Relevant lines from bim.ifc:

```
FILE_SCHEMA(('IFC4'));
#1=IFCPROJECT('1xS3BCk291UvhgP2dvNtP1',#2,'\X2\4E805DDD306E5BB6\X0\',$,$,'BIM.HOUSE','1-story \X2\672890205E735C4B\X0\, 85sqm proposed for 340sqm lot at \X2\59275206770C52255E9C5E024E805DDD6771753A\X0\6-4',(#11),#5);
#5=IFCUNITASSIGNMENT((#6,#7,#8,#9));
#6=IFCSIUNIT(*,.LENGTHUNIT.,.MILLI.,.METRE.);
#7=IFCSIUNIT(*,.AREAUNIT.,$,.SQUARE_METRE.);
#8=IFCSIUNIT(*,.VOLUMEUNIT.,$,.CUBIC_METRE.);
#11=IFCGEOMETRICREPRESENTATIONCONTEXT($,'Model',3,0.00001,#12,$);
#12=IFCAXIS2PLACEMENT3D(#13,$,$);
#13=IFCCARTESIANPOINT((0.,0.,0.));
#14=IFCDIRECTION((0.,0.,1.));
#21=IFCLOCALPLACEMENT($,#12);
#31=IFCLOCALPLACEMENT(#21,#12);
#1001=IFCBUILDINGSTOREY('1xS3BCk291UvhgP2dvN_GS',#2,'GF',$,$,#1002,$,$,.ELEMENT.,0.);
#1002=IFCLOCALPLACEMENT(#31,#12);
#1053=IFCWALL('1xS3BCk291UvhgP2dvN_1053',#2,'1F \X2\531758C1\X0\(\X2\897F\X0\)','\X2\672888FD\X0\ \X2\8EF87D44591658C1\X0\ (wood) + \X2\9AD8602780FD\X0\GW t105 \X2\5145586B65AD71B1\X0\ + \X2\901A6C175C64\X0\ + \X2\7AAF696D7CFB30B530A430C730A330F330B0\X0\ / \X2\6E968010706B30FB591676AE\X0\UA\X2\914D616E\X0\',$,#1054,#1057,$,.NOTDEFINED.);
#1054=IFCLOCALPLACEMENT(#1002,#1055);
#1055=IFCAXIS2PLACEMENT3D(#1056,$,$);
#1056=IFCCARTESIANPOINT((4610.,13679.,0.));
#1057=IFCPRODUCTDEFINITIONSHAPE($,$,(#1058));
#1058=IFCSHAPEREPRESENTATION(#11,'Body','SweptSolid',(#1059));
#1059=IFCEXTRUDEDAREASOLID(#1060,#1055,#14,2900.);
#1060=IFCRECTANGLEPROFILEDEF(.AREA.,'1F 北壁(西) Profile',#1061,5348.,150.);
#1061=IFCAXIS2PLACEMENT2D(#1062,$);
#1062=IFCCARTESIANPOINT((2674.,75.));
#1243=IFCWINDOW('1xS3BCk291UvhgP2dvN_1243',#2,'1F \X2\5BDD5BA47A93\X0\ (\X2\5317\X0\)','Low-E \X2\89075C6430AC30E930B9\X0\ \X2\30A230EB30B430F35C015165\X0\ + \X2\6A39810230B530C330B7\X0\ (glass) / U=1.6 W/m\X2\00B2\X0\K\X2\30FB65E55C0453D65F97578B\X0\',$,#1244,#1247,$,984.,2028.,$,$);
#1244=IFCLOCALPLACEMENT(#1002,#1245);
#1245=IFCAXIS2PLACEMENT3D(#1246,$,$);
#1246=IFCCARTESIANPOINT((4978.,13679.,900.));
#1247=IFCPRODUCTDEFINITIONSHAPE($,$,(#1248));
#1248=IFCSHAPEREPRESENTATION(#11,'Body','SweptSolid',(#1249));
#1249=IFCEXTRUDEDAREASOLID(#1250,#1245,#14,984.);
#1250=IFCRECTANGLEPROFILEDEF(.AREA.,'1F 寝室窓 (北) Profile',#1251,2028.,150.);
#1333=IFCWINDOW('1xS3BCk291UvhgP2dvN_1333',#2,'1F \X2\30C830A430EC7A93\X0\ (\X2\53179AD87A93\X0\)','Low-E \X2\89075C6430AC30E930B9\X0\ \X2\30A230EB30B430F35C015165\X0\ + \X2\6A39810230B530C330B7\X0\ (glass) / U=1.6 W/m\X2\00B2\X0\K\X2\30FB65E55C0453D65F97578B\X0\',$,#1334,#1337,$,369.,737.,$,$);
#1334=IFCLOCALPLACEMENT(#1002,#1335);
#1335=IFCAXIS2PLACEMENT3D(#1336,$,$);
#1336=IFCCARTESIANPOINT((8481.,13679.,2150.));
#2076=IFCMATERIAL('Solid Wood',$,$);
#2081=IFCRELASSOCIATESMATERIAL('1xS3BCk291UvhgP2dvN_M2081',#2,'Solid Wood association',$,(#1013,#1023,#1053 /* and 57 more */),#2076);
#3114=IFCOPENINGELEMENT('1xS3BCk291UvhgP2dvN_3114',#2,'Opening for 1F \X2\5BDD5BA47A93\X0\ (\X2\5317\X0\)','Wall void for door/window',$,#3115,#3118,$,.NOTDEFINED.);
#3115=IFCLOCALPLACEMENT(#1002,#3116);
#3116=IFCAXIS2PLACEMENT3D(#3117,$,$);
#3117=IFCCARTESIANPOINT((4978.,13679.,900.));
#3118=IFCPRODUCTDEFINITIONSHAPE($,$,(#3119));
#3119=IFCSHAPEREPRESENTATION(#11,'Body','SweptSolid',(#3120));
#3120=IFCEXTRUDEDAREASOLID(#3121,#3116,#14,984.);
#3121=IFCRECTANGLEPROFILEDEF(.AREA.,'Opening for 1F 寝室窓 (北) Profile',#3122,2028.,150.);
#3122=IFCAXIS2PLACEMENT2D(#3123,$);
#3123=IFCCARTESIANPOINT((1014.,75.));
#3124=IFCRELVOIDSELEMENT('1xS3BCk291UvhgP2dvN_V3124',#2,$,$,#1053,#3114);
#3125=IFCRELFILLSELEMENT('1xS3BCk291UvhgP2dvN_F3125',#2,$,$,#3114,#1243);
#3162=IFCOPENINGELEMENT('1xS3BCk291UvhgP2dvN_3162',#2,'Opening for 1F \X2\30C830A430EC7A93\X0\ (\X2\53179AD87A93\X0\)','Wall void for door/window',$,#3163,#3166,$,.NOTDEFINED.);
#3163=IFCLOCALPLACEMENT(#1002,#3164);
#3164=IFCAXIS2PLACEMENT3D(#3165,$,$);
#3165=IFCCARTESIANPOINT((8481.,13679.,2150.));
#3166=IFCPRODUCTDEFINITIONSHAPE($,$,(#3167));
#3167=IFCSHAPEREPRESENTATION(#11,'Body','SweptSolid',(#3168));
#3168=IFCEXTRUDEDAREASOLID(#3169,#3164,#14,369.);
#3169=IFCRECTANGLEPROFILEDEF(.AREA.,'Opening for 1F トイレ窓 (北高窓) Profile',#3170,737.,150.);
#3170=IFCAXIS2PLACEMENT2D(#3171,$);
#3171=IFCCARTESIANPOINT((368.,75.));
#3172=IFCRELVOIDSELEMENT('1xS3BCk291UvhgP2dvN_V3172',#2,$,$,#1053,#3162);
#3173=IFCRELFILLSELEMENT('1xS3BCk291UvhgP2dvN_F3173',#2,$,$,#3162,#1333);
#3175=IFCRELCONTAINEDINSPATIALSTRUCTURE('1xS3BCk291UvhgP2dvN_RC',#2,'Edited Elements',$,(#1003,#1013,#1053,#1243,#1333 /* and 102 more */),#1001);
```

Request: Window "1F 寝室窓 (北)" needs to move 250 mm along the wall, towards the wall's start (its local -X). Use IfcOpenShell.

```python
import ifcopenshell
import ifcopenshell.api.geometry
import ifcopenshell.util.placement

model = ifcopenshell.open("bim.ifc")

window = model.by_guid("1xS3BCk291UvhgP2dvN_1243")
opening = window.FillsVoids[0].RelatingOpeningElement
wall = opening.VoidsElements[0].RelatingBuildingElement

wall_matrix = ifcopenshell.util.placement.get_local_placement(wall.ObjectPlacement)
shift = wall_matrix[:3, 0] * -250.0
before = ifcopenshell.util.placement.get_local_placement(window.ObjectPlacement)[:3, 3].copy()

# The window is not placed relative to its opening, so move both.
for product in (opening, window):
    matrix = ifcopenshell.util.placement.get_local_placement(product.ObjectPlacement)
    matrix[:3, 3] += shift
    ifcopenshell.api.geometry.edit_object_placement(model, product=product, matrix=matrix, is_si=False)

after = ifcopenshell.util.placement.get_local_placement(window.ObjectPlacement)[:3, 3]
print("window moved by", (after - before).round(3) + 0.0)

model.write("bim_v2.ifc")
```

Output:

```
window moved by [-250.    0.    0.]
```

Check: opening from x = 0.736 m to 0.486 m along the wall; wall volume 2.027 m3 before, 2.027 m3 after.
